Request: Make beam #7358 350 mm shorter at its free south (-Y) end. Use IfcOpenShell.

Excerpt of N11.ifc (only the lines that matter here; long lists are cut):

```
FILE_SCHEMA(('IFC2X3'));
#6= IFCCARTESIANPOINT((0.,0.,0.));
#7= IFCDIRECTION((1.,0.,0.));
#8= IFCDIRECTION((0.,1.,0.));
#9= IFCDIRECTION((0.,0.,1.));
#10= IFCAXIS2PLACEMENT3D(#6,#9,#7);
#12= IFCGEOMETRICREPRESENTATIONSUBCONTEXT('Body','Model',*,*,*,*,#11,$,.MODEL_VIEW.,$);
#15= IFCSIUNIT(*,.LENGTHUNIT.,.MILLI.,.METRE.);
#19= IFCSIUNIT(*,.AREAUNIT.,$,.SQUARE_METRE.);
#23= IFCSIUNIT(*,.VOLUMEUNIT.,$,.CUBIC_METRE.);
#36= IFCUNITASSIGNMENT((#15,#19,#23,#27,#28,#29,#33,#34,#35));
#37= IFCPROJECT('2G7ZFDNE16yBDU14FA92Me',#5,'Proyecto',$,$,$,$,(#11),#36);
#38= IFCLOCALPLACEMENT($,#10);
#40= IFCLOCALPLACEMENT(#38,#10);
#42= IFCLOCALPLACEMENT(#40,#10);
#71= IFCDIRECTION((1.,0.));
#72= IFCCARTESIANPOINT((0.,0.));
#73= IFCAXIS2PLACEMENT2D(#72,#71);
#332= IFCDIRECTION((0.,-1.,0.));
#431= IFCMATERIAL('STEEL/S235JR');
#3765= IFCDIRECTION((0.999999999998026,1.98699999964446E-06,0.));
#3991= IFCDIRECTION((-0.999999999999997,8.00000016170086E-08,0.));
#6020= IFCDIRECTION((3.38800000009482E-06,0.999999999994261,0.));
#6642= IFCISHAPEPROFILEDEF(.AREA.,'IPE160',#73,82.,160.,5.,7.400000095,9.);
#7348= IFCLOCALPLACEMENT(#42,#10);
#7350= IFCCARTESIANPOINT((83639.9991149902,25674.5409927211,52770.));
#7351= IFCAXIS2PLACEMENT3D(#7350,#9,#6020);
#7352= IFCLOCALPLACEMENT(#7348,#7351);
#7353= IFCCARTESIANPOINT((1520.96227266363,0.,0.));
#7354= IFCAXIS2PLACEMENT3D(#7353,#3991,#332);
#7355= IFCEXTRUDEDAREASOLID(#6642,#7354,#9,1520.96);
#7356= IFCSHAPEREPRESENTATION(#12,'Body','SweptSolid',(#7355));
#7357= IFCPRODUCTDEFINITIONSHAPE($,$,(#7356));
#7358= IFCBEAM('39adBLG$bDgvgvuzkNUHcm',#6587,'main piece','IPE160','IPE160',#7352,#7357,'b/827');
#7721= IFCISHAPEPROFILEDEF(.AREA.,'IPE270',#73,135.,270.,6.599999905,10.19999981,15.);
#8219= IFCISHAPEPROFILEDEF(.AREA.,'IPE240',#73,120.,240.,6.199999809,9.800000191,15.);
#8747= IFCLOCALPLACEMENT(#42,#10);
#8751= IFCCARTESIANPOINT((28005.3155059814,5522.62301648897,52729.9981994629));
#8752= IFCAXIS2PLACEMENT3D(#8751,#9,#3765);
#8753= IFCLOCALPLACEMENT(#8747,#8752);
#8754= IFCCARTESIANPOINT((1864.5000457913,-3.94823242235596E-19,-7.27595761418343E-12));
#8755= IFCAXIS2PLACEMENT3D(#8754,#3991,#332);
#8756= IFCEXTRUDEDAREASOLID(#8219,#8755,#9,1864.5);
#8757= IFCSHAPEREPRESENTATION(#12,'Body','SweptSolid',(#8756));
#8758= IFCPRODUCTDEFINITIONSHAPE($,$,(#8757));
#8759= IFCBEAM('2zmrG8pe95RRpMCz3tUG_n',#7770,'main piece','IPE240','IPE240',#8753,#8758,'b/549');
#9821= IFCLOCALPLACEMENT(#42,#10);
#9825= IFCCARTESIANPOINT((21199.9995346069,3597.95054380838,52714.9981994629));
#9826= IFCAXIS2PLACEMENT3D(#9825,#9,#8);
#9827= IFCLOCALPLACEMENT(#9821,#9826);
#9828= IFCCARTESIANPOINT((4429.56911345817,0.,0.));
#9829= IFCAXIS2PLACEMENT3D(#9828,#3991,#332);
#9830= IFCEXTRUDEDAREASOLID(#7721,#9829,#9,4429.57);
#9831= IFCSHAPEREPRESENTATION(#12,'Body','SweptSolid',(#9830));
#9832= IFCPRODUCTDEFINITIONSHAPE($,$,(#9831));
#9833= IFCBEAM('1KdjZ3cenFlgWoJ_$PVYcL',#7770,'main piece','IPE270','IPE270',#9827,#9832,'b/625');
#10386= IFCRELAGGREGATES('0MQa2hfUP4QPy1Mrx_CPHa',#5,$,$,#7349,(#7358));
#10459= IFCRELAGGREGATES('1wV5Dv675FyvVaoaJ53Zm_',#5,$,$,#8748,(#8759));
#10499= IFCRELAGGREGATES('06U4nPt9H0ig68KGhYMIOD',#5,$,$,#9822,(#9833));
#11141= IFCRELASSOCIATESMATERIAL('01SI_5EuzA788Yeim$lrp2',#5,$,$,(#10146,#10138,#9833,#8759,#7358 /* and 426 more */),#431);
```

```python
import ifcopenshell
import ifcopenshell.util.representation

model = ifcopenshell.open("N11.ifc")

member = model.by_id(7358)
change = -350.0

# The extrusion runs towards the end named, so only its depth changes.
body = ifcopenshell.util.representation.get_representation(member, "Model", "Body")
solid = body.Items[0]
old_length = solid.Depth
solid.Depth += change

print(f"length {old_length:g} -> {solid.Depth:g}")

model.write("N11_edited.ifc")
```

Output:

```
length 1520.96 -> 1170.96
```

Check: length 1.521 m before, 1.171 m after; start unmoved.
